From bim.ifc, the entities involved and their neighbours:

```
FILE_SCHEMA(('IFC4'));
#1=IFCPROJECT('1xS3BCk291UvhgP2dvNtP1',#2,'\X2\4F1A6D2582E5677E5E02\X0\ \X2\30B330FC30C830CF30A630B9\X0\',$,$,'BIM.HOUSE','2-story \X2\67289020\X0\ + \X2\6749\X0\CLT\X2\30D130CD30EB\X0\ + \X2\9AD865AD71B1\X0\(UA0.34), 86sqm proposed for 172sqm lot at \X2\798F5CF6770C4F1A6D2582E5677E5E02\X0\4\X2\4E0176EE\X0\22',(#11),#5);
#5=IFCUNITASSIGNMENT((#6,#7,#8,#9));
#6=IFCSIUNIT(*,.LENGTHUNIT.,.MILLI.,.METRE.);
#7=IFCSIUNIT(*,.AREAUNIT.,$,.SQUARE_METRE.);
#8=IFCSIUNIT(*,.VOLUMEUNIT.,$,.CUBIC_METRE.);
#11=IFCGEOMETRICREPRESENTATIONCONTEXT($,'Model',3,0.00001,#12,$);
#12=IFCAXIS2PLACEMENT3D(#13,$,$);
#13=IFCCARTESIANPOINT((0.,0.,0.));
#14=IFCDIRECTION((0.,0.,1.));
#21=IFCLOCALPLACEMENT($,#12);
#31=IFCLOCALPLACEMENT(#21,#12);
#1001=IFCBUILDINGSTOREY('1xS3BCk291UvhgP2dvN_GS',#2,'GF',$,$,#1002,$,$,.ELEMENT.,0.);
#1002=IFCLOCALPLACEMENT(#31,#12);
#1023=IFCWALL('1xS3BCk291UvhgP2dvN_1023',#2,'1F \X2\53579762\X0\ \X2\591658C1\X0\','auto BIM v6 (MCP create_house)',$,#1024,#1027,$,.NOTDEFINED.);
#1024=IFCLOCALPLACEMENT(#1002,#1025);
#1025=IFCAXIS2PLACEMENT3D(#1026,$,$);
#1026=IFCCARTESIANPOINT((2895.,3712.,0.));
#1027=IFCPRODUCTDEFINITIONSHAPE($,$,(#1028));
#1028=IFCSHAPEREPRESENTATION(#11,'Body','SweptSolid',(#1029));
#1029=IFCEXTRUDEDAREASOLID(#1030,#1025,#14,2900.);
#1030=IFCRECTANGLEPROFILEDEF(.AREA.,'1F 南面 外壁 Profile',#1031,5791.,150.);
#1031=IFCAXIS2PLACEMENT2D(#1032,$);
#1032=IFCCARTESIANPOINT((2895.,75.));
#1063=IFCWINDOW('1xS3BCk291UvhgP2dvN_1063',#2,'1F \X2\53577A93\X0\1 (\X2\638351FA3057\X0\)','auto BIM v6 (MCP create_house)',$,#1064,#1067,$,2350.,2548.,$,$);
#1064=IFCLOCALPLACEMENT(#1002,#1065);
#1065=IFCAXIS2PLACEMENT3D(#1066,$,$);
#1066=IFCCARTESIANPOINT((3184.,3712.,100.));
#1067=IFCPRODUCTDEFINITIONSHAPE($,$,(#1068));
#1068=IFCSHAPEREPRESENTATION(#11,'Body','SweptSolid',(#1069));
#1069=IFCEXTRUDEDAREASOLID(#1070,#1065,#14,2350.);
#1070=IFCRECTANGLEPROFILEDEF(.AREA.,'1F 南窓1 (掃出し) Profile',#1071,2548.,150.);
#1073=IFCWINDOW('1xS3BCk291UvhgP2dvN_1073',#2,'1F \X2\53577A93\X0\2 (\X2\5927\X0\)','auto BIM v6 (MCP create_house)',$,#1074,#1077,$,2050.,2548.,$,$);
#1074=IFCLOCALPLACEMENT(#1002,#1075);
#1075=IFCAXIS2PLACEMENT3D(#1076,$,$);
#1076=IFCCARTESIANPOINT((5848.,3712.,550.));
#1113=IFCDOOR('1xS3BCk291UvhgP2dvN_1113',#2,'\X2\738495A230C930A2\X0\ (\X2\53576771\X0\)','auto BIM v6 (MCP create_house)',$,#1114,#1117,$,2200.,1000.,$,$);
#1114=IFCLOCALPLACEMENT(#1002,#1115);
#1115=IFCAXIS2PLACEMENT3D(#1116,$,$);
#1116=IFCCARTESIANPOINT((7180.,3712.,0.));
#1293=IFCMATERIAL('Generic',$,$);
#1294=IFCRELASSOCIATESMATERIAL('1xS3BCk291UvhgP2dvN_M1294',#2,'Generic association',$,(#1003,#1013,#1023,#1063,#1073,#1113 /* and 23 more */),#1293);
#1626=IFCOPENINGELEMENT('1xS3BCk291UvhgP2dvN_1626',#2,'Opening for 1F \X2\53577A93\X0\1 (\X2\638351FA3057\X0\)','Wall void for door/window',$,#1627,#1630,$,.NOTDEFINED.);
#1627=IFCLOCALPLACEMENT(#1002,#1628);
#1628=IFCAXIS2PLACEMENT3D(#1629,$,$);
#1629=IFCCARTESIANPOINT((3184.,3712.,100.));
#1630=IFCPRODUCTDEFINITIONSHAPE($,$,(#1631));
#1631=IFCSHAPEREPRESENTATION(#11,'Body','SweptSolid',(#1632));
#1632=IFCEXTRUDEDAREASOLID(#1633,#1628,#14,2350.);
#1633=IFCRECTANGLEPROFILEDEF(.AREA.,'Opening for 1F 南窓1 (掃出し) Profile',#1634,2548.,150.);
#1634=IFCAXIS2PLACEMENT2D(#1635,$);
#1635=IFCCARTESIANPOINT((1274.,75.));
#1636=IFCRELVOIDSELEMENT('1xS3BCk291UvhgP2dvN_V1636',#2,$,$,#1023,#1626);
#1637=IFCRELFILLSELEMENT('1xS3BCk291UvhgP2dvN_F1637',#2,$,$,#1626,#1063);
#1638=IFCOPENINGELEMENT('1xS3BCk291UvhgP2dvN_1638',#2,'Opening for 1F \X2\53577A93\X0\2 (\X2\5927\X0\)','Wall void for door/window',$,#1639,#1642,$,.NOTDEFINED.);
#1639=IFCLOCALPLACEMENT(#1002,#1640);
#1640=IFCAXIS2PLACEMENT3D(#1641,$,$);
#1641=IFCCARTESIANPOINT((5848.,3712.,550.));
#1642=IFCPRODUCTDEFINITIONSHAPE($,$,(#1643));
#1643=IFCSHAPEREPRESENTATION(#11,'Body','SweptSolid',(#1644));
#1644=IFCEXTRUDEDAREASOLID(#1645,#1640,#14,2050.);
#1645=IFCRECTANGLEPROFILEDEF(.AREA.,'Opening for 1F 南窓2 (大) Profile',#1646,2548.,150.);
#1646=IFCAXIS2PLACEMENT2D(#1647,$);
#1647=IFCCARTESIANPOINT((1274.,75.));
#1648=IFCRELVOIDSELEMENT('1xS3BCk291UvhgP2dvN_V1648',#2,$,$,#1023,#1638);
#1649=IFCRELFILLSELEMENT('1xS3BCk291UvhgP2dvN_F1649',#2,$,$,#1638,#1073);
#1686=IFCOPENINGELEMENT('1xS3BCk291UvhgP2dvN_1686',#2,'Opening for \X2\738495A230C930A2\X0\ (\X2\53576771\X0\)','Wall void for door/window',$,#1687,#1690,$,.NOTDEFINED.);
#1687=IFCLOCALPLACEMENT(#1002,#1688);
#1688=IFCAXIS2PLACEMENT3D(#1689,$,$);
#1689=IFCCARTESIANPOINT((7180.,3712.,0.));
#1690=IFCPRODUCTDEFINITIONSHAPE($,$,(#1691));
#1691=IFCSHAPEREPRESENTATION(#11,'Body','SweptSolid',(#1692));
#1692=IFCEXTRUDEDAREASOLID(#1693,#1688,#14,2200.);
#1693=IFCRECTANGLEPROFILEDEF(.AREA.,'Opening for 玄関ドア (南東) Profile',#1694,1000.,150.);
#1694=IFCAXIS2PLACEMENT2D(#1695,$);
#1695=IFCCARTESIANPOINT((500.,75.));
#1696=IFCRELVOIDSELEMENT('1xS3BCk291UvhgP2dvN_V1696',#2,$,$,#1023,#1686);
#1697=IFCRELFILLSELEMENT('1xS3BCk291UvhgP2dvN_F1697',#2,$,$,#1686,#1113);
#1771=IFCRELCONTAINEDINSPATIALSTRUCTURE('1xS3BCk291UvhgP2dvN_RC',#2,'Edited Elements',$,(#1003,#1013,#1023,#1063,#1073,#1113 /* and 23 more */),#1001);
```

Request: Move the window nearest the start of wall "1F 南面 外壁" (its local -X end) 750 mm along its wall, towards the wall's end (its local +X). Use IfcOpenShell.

```python
import ifcopenshell
import ifcopenshell.api.geometry
import ifcopenshell.util.placement

model = ifcopenshell.open("bim.ifc")

window = model.by_guid("1xS3BCk291UvhgP2dvN_1063")
opening = window.FillsVoids[0].RelatingOpeningElement
wall = opening.VoidsElements[0].RelatingBuildingElement

wall_matrix = ifcopenshell.util.placement.get_local_placement(wall.ObjectPlacement)
shift = wall_matrix[:3, 0] * 750.0
before = ifcopenshell.util.placement.get_local_placement(window.ObjectPlacement)[:3, 3].copy()

# The window is not placed relative to its opening, so move both.
for product in (opening, window):
    matrix = ifcopenshell.util.placement.get_local_placement(product.ObjectPlacement)
    matrix[:3, 3] += shift
    ifcopenshell.api.geometry.edit_object_placement(model, product=product, matrix=matrix, is_si=False)

after = ifcopenshell.util.placement.get_local_placement(window.ObjectPlacement)[:3, 3]
print("window moved by", (after - before).round(3) + 0.0)

model.write("bim_v2.ifc")
```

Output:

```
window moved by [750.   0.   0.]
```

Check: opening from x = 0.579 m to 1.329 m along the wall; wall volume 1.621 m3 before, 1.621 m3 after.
